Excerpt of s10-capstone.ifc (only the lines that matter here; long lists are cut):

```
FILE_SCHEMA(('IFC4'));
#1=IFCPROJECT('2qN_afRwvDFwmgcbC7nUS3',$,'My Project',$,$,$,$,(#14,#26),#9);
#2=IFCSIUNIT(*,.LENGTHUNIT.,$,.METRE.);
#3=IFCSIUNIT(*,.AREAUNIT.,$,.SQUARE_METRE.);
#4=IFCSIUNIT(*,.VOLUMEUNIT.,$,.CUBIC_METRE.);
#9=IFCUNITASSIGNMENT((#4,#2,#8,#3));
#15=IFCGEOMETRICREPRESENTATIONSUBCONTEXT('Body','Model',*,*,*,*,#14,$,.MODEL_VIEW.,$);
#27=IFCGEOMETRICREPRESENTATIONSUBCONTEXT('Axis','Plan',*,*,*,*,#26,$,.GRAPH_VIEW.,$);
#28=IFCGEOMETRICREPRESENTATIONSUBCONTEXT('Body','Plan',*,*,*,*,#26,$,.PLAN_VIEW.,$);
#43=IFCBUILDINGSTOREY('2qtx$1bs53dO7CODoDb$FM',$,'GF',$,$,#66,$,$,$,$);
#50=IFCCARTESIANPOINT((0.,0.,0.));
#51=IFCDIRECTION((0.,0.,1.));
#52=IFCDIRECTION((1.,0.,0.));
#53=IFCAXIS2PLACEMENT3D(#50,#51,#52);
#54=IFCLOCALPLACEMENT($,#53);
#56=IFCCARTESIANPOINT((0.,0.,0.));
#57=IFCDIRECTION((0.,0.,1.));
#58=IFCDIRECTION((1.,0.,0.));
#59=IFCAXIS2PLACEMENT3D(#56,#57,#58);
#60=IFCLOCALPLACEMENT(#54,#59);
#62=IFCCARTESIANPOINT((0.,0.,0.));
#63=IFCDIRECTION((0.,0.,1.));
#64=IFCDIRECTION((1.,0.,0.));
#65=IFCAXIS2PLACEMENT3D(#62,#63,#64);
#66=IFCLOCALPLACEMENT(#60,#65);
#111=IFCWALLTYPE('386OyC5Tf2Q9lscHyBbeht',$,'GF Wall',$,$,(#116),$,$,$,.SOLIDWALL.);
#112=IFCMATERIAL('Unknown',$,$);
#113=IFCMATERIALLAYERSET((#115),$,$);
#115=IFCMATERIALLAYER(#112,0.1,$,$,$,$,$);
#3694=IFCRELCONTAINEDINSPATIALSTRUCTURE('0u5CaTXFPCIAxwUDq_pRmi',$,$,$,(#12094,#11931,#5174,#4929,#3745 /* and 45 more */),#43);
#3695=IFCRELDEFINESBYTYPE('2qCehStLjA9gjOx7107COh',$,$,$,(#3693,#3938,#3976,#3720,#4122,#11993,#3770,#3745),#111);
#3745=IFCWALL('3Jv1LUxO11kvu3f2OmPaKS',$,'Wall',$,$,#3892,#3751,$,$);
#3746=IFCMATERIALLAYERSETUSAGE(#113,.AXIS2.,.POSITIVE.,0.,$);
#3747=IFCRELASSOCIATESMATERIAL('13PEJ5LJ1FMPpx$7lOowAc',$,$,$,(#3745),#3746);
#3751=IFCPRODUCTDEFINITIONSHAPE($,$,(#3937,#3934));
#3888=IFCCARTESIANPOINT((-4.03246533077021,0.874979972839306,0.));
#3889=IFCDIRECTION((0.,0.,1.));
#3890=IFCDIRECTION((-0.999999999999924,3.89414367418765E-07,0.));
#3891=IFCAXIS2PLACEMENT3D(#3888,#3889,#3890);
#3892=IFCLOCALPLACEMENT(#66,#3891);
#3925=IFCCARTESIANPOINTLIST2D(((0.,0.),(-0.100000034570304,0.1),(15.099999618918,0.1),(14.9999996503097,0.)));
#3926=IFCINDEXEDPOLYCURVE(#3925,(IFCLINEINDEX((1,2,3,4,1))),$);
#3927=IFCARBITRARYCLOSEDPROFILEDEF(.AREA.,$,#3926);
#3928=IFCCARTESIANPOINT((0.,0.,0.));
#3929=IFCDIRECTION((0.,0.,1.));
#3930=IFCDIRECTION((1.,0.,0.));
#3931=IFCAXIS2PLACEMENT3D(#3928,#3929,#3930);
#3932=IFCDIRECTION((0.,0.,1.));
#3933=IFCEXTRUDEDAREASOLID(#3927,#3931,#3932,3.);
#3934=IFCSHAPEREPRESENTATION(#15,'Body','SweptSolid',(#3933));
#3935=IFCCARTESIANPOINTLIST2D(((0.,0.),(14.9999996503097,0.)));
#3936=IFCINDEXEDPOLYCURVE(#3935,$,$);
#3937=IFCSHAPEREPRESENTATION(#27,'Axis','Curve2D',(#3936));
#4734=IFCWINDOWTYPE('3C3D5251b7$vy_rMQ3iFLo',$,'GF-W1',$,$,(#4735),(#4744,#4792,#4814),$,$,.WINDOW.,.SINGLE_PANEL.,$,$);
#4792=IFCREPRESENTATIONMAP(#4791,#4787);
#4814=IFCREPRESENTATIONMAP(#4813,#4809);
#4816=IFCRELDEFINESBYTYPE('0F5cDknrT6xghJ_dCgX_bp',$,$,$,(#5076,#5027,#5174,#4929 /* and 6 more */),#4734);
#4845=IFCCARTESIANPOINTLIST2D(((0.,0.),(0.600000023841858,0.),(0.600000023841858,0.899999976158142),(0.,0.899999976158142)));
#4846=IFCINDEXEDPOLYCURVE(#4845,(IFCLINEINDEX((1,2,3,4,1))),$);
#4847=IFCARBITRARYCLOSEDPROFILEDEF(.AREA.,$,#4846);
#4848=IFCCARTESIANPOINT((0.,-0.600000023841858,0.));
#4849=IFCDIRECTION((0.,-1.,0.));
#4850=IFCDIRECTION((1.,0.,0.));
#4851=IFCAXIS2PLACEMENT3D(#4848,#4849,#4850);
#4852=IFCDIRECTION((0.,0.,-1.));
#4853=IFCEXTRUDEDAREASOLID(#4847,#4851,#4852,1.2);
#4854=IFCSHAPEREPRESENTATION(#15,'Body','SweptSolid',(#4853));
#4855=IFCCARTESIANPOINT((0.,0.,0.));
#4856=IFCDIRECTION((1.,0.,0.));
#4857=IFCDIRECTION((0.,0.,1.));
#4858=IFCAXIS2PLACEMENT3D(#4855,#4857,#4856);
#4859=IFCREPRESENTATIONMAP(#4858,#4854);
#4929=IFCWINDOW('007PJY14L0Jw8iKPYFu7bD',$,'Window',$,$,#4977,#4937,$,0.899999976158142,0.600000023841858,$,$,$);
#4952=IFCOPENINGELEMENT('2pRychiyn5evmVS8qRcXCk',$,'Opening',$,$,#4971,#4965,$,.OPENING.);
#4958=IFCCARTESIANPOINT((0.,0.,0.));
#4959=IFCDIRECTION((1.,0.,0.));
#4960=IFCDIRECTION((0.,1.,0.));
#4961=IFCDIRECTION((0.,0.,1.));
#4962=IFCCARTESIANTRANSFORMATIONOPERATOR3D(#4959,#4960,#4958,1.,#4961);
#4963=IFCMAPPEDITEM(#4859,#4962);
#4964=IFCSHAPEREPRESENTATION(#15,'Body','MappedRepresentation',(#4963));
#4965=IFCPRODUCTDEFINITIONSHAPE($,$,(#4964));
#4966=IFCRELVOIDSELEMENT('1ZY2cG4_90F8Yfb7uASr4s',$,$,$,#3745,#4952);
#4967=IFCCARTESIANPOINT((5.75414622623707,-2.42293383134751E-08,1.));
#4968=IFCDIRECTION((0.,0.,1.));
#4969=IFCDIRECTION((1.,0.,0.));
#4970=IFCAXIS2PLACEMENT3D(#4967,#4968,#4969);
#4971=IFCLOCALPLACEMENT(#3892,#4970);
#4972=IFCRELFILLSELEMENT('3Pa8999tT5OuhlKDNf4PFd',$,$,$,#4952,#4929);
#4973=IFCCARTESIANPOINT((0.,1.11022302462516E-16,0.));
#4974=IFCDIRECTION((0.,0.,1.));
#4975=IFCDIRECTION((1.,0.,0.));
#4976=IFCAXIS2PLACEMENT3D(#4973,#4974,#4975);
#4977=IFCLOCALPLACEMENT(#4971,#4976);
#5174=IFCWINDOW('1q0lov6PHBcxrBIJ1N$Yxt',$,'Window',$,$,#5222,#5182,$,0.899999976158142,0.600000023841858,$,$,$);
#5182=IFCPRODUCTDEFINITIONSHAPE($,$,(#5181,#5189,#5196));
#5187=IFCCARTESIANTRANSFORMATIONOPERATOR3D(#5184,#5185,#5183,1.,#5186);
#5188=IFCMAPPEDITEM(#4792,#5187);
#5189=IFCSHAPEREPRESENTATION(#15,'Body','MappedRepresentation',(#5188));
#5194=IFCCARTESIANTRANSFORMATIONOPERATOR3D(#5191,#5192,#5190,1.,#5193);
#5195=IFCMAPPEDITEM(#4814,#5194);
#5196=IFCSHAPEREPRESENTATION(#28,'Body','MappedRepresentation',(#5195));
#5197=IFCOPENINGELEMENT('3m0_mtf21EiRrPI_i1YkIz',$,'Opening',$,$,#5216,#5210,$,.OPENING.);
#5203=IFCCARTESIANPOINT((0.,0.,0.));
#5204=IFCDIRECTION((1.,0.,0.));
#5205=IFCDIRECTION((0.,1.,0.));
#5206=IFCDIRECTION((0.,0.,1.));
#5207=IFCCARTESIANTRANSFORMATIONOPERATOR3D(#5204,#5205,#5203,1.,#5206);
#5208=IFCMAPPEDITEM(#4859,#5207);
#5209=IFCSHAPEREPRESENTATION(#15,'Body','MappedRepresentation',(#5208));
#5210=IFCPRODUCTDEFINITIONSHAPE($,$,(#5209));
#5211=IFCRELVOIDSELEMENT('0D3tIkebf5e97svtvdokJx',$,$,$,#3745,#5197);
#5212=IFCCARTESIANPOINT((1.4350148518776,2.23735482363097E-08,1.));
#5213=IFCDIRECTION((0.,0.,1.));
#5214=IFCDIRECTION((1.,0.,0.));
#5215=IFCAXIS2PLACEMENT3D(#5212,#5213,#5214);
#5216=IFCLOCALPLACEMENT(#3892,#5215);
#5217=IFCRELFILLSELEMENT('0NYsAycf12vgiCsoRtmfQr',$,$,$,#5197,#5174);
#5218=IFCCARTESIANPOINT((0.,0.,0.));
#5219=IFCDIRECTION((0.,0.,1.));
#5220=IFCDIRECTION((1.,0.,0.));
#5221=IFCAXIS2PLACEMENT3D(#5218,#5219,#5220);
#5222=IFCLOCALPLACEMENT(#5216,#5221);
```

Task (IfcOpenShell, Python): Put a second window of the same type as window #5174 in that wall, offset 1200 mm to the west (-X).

```python
import ifcopenshell
import ifcopenshell.api.feature
import ifcopenshell.api.geometry
import ifcopenshell.api.root
import ifcopenshell.geom
import ifcopenshell.util.element
import ifcopenshell.util.placement
import ifcopenshell.util.shape
import ifcopenshell.util.unit

model = ifcopenshell.open("s10-capstone.ifc")
unit_scale = ifcopenshell.util.unit.calculate_unit_scale(model)
settings = ifcopenshell.geom.settings()


def volume(element):
    """Net volume in cubic metres, openings subtracted."""
    shape = ifcopenshell.geom.create_shape(settings, element)
    return ifcopenshell.util.shape.get_volume(shape.geometry)


window = model.by_guid("1q0lov6PHBcxrBIJ1N$Yxt")
opening = window.FillsVoids[0].RelatingOpeningElement
wall = opening.VoidsElements[0].RelatingBuildingElement
before = volume(wall)
shift = ifcopenshell.util.placement.get_local_placement(wall.ObjectPlacement)[:3, 0] * 1.2 / unit_scale

# copy_class copies the void relationship, type, container and properties, but no geometry.
new_opening = ifcopenshell.api.root.copy_class(model, product=opening)
new_opening.Representation = ifcopenshell.util.element.copy_deep(
    model, opening.Representation, exclude=["IfcGeometricRepresentationContext", "IfcRepresentationMap"]
)
new_window = ifcopenshell.api.root.copy_class(model, product=window)
new_window.Representation = ifcopenshell.util.element.copy_deep(
    model, window.Representation, exclude=["IfcGeometricRepresentationContext", "IfcRepresentationMap"]
)
ifcopenshell.api.feature.add_filling(model, opening=new_opening, element=new_window)

for old, new in ((opening, new_opening), (window, new_window)):
    matrix = ifcopenshell.util.placement.get_local_placement(old.ObjectPlacement)
    matrix[:3, 3] += shift
    ifcopenshell.api.geometry.edit_object_placement(model, product=new, matrix=matrix, is_si=False)

after = volume(wall)

print(f"wall volume {before:.3f} -> {after:.3f} m3")

model.write("s10-capstone_updated.ifc")
```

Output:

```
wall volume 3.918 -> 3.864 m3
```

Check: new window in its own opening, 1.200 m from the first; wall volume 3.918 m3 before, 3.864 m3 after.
